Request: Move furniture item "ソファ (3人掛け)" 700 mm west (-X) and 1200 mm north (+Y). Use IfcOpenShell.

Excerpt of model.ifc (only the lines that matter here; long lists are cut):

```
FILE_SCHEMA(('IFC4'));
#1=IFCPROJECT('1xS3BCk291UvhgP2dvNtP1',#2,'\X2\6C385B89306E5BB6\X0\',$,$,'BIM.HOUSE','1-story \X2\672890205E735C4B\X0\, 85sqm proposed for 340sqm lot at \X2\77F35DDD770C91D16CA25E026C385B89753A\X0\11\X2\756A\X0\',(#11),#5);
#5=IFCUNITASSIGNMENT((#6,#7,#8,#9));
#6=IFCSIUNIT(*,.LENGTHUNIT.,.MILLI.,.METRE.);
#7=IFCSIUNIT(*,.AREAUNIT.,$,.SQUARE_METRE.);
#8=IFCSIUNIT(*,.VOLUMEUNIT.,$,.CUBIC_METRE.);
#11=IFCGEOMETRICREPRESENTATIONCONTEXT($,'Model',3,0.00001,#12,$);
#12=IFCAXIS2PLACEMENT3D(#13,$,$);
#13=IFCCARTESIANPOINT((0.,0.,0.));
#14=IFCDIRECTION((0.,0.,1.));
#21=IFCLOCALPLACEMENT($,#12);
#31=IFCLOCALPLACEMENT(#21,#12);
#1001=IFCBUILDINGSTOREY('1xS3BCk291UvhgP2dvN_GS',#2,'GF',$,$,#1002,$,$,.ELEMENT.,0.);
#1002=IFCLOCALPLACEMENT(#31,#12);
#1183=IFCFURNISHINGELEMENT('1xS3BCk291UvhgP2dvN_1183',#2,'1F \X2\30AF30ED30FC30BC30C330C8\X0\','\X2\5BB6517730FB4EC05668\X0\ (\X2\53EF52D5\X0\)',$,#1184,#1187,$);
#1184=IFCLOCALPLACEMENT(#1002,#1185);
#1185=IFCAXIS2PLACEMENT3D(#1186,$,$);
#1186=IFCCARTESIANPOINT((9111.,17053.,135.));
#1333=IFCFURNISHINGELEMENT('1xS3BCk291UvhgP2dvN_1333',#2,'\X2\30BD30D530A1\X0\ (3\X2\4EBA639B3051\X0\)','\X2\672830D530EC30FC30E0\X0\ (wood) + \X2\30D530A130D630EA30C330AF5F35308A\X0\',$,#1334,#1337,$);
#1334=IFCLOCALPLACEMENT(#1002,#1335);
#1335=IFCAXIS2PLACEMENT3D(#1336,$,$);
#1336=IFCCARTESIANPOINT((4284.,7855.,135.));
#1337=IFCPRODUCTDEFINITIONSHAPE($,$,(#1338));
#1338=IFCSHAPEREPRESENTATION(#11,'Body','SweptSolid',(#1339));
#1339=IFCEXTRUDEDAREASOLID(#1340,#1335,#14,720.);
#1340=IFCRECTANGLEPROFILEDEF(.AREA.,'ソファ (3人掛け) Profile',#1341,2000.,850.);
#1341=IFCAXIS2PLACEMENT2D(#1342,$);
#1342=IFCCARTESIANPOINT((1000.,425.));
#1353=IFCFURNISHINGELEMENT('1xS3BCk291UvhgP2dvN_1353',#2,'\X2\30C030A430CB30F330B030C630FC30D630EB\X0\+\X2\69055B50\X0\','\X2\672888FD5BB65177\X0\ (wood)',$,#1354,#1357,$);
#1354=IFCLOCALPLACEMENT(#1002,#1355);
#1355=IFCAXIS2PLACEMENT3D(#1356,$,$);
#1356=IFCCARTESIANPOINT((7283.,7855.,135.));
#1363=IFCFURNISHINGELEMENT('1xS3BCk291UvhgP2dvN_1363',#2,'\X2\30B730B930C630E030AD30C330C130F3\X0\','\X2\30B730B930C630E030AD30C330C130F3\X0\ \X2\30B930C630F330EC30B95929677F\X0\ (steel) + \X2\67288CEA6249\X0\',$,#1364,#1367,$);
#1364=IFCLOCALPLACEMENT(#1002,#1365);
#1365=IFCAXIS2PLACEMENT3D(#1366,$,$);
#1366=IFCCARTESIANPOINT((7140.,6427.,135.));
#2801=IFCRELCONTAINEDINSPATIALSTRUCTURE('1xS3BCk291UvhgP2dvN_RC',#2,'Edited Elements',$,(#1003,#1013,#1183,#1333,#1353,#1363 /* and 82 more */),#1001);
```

```python
import ifcopenshell
import ifcopenshell.api.geometry
import ifcopenshell.util.placement
import ifcopenshell.util.unit

model = ifcopenshell.open("model.ifc")
unit_scale = ifcopenshell.util.unit.calculate_unit_scale(model)

item = model.by_guid("1xS3BCk291UvhgP2dvN_1333")
matrix = ifcopenshell.util.placement.get_local_placement(item.ObjectPlacement)
matrix[0, 3] -= 0.7 / unit_scale
matrix[1, 3] += 1.2 / unit_scale
ifcopenshell.api.geometry.edit_object_placement(model, product=item, matrix=matrix, is_si=False)

print(ifcopenshell.util.placement.get_local_placement(item.ObjectPlacement).round(3) + 0.0)

model.write("model_updated.ifc")
```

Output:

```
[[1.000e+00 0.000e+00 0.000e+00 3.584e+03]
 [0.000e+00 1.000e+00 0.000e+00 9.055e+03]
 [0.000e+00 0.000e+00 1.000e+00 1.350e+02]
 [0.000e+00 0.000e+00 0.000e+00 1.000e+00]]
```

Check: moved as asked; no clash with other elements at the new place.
